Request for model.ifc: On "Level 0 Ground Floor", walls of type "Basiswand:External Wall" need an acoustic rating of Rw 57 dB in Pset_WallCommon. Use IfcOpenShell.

First a look at what the model holds.

```python
import ifcopenshell
import ifcopenshell.util.element

model = ifcopenshell.open("model.ifc")
print(model.schema)
storey = next(s for s in model.by_type("IfcBuildingStorey") if s.Name == "Level 0 Ground Floor")
walls = [e for e in ifcopenshell.util.element.get_decomposition(storey) if e.is_a("IfcWall")]
seen = {}
for e in walls:
    element_type = ifcopenshell.util.element.get_type(e)
    key = (element_type.Name if element_type != e and element_type else None, ifcopenshell.util.element.get_pset(e, "Pset_WallCommon", "AcousticRating"))
    seen[key] = seen.get(key, 0) + 1
for (name, value), count in sorted(seen.items(), key=str):
    print(count, "x", name, "|", value)
```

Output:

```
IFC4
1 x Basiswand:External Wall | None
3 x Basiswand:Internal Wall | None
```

```python
import ifcopenshell
import ifcopenshell.api.pset
import ifcopenshell.util.element

model = ifcopenshell.open("model.ifc")

storey = next(s for s in model.by_type("IfcBuildingStorey") if s.Name == "Level 0 Ground Floor")
walls = [e for e in ifcopenshell.util.element.get_decomposition(storey) if e.is_a("IfcWall")]

count = 0
for e in walls:
    element_type = ifcopenshell.util.element.get_type(e)
    if element_type in (None, e) or element_type.Name != "Basiswand:External Wall":
        continue
    # add_pset returns the element's existing set when there is one.
    pset = ifcopenshell.api.pset.add_pset(model, product=e, name="Pset_WallCommon")
    ifcopenshell.api.pset.edit_pset(model, pset=pset, properties={"AcousticRating": "Rw 57 dB"})
    count += 1

print(count, "walls updated")

model.write("model_rev.ifc")
```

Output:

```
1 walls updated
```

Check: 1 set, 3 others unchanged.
